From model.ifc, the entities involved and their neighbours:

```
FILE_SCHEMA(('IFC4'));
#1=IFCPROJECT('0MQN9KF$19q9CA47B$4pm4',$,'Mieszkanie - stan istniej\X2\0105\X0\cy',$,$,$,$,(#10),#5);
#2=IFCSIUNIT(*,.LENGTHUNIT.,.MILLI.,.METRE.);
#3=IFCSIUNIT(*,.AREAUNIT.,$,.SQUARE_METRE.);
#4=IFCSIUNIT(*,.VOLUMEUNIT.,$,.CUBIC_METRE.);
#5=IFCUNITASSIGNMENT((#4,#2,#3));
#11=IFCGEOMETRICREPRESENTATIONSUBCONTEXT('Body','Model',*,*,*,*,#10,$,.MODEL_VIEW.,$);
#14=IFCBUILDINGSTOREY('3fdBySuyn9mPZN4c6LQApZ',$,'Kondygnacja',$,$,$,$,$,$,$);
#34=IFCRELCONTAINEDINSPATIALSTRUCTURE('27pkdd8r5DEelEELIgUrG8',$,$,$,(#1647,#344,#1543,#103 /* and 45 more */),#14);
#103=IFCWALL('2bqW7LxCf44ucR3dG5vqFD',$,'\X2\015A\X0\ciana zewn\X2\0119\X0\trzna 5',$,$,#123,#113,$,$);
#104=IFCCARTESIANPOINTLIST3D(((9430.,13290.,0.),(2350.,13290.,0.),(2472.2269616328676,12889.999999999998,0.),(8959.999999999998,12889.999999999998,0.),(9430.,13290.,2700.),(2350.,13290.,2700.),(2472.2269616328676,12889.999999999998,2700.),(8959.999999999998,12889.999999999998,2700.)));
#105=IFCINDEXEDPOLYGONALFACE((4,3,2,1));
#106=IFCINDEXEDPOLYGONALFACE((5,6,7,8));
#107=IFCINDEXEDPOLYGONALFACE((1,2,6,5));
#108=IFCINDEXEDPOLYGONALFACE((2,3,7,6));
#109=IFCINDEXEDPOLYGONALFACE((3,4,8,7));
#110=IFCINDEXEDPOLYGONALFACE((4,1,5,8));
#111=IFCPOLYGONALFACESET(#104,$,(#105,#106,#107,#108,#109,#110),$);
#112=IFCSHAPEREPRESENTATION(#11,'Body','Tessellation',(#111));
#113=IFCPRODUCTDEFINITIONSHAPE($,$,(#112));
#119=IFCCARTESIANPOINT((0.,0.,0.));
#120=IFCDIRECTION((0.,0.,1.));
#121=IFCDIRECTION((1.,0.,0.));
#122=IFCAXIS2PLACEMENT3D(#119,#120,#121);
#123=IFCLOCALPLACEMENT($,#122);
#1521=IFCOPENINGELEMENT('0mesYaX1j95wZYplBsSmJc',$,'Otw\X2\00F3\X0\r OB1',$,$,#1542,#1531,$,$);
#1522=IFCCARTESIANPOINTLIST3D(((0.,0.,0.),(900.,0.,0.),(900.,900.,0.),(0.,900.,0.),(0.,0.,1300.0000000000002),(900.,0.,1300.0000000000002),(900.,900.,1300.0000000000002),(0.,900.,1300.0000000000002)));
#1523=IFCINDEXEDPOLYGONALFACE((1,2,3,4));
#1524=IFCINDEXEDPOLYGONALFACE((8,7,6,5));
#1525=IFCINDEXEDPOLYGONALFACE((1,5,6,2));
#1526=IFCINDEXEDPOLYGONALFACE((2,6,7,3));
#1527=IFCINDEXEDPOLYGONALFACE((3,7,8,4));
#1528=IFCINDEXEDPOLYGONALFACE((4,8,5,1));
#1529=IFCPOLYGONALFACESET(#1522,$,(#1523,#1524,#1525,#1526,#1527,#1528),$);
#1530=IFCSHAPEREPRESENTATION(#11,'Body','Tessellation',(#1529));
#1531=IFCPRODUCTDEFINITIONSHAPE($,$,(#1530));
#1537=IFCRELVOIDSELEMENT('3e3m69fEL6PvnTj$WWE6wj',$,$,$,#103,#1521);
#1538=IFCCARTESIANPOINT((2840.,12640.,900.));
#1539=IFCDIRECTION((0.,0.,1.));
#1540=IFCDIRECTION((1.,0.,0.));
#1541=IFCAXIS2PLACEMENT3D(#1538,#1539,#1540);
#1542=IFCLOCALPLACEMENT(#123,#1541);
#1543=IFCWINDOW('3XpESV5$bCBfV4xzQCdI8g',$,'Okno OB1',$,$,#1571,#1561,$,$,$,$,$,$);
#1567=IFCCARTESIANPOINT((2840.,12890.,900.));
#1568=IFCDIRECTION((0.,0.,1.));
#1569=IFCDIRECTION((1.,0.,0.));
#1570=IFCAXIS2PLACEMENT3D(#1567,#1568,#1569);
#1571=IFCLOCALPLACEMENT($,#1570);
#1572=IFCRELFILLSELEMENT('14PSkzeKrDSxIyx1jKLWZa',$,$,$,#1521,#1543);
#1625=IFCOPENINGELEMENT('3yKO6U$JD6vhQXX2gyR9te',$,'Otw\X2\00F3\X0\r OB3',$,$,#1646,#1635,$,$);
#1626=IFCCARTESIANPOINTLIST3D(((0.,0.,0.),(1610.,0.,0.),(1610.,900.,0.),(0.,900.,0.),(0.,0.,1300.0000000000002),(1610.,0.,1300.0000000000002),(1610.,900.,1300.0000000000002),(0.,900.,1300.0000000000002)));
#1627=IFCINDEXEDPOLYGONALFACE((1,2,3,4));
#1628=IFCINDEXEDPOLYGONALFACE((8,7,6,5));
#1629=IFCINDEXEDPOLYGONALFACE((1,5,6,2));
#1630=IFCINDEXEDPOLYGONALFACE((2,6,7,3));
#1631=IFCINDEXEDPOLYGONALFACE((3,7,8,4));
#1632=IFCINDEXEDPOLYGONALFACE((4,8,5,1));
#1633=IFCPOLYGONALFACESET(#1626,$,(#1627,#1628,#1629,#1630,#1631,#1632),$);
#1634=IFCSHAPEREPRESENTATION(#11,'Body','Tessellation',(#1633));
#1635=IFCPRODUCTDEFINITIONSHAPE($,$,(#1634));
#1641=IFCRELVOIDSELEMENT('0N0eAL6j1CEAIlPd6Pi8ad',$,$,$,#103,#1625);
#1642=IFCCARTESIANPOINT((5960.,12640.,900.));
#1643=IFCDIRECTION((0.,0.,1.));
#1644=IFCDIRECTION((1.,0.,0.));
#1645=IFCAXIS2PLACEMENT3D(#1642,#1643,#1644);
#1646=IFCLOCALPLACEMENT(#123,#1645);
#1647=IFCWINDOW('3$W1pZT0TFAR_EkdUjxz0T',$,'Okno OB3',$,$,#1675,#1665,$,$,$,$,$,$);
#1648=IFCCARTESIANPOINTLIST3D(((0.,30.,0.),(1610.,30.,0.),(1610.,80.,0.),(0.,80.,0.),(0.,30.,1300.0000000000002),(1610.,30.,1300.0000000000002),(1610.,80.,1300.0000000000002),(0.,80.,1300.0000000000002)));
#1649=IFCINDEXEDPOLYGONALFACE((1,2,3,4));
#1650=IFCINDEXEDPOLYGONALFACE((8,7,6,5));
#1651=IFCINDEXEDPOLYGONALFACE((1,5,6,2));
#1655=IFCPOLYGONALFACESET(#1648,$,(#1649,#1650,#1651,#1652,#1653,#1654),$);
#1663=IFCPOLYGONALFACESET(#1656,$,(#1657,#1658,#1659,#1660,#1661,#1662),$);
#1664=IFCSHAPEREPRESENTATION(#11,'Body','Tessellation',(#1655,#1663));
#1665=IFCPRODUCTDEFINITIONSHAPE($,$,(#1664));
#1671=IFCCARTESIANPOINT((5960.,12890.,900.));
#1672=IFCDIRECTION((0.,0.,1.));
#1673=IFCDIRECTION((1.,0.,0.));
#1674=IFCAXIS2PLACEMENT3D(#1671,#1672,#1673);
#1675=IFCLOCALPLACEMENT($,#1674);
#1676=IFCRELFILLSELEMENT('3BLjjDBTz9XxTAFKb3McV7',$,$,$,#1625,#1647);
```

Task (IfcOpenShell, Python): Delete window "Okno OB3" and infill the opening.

```python
import ifcopenshell
import ifcopenshell.api.feature
import ifcopenshell.api.root
import ifcopenshell.geom
import ifcopenshell.util.shape

model = ifcopenshell.open("model.ifc")
settings = ifcopenshell.geom.settings()


def volume(element):
    """Net volume in cubic metres, openings subtracted."""
    shape = ifcopenshell.geom.create_shape(settings, element)
    return ifcopenshell.util.shape.get_volume(shape.geometry)


window = model.by_guid("3$W1pZT0TFAR_EkdUjxz0T")
opening = window.FillsVoids[0].RelatingOpeningElement
wall = opening.VoidsElements[0].RelatingBuildingElement
before = volume(wall)

ifcopenshell.api.root.remove_product(model, product=window)
ifcopenshell.api.feature.remove_feature(model, feature=opening)

after = volume(wall)

print(f"wall volume {before:.3f} -> {after:.3f} m3")

model.write("model_rev.ifc")
```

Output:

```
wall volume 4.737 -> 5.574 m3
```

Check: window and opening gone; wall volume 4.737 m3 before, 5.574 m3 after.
